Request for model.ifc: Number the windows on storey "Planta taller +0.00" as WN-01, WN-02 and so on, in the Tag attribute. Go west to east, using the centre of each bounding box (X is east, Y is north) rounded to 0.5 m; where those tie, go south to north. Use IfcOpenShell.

First a look at what the model holds.

```python
import ifcopenshell
import ifcopenshell.util.element
import ifcopenshell.util.placement

model = ifcopenshell.open("model.ifc")
print(model.schema)
storey = next(s for s in model.by_type("IfcBuildingStorey") if s.Name == "Planta taller +0.00")
windows = [e for e in ifcopenshell.util.element.get_decomposition(storey) if e.is_a("IfcWindow")]
for e in sorted(windows, key=lambda e: e.id()):
    origin = ifcopenshell.util.placement.get_local_placement(e.ObjectPlacement)[:3, 3]
    print(e.id(), e.Tag, e.Name, origin.round(2) + 0.0, sep=" | ")
```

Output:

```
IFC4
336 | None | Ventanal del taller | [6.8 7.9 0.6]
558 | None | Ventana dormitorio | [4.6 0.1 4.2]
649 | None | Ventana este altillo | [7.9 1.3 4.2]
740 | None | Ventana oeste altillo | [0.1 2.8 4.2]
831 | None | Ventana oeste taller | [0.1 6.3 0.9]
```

```python
import ifcopenshell
import ifcopenshell.geom
import ifcopenshell.util.element
import ifcopenshell.util.shape

model = ifcopenshell.open("model.ifc")
settings = ifcopenshell.geom.settings()
settings.set("use-world-coords", True)


def centre(element):
    shape = ifcopenshell.geom.create_shape(settings, element)
    return ifcopenshell.util.shape.get_bbox_centroid(shape.geometry)


storey = next(s for s in model.by_type("IfcBuildingStorey") if s.Name == "Planta taller +0.00")
windows = [e for e in ifcopenshell.util.element.get_decomposition(storey) if e.is_a("IfcWindow")]

# Insertion points can sit at a corner or the storey origin, so sort by the geometry (in metres).
centres = {e: centre(e) for e in windows}
windows.sort(key=lambda e: (round(centres[e][0] / 0.5), centres[e][1]))

for i, e in enumerate(windows, start=1):
    number = f"WN-{i:02d}"
    e.Tag = number
    print(e.id(), number)

model.write("model-out.ifc")
```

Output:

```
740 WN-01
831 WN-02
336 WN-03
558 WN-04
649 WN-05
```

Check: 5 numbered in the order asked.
